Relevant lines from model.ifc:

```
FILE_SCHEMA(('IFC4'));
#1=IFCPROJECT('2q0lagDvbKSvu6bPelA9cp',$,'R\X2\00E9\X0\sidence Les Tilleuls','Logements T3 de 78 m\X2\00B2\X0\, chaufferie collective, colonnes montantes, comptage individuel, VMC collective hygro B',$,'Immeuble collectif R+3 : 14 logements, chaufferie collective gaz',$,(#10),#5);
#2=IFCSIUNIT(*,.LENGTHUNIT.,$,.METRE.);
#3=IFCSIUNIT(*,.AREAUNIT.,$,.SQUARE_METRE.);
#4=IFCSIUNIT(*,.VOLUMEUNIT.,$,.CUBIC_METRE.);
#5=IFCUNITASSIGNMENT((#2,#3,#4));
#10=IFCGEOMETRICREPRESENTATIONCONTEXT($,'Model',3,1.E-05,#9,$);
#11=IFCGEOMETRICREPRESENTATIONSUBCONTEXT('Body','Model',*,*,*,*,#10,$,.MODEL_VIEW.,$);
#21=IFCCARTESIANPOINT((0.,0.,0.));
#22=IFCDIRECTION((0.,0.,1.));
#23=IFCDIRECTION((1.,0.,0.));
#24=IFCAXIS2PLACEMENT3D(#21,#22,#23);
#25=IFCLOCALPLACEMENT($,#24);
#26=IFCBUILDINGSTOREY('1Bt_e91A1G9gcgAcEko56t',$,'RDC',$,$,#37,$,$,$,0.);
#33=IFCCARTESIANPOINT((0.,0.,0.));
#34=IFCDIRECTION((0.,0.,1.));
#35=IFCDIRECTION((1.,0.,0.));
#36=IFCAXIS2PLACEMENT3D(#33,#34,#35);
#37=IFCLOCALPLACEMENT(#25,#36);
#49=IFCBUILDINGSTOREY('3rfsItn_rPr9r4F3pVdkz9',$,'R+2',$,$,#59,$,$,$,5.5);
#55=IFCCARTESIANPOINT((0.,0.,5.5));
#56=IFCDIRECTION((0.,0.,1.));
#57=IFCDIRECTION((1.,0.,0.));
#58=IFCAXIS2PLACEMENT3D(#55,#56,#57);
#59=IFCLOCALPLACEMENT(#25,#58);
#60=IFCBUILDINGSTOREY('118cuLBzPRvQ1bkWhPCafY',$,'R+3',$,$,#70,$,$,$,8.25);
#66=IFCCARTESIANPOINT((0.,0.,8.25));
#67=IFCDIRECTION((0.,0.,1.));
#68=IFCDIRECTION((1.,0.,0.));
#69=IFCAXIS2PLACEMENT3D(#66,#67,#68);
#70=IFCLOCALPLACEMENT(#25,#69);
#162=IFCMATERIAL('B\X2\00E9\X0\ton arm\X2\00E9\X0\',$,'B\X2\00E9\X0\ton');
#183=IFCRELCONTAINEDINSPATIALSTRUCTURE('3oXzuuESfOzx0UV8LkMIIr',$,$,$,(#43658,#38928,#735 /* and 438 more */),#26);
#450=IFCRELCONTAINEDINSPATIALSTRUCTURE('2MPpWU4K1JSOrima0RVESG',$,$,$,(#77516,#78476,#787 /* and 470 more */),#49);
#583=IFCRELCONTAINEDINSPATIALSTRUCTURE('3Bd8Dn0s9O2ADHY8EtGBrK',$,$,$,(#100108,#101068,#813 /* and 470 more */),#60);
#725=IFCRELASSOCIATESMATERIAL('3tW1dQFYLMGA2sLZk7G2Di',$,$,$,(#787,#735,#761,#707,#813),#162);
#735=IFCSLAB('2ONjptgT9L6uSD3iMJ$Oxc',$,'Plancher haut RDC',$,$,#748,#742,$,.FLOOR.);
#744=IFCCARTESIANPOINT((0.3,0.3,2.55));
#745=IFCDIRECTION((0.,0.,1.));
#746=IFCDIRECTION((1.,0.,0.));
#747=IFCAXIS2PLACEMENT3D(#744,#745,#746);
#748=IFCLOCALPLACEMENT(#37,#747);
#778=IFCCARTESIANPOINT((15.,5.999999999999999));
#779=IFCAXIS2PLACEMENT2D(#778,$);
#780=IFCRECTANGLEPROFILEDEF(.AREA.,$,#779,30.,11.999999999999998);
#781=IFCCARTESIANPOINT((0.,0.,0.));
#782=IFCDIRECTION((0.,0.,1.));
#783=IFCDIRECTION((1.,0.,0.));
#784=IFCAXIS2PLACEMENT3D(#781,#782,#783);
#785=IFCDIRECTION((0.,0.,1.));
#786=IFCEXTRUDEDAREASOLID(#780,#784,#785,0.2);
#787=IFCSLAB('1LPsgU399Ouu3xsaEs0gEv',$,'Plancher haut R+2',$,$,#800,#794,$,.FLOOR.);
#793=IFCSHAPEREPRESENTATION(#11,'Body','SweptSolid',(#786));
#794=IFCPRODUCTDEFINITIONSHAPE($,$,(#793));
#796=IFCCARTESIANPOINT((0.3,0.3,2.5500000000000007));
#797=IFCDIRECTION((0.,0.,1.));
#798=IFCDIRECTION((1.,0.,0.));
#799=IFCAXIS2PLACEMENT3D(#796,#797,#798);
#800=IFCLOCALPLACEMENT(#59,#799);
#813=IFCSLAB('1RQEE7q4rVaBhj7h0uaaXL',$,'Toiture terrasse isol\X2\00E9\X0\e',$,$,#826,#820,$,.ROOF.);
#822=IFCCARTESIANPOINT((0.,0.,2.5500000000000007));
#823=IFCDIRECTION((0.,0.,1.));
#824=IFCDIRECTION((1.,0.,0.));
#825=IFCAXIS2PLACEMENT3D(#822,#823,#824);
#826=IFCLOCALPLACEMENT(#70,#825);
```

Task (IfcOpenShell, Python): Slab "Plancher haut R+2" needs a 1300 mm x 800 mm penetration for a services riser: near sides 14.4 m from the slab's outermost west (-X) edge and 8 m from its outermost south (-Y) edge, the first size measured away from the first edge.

```python
import numpy as np
import ifcopenshell
import ifcopenshell.api.feature
import ifcopenshell.api.geometry
import ifcopenshell.api.root
import ifcopenshell.geom
import ifcopenshell.util.placement
import ifcopenshell.util.representation
import ifcopenshell.util.shape
import ifcopenshell.util.unit

model = ifcopenshell.open("model.ifc")
unit_scale = ifcopenshell.util.unit.calculate_unit_scale(model)
settings = ifcopenshell.geom.settings()


def volume(element):
    """Net volume in cubic metres, openings subtracted."""
    shape = ifcopenshell.geom.create_shape(settings, element)
    return ifcopenshell.util.shape.get_volume(shape.geometry)


slab = model.by_id(787)
before = volume(slab)

# Extent in the slab's own axes, in metres. The edges named are its -X and -Y sides.
slab_shape = ifcopenshell.geom.create_shape(settings, slab)
vertices = ifcopenshell.util.shape.get_vertices(slab_shape.geometry)
x_min, y_min, bottom = vertices.min(axis=0)
top = vertices[:, 2].max()

opening = ifcopenshell.api.root.create_entity(model, ifc_class="IfcOpeningElement", name="Services riser opening", predefined_type="OPENING")
context = ifcopenshell.util.representation.get_context(model, "Model", "Body", "MODEL_VIEW")
width, depth = 1.3, 0.8
outline = [(0.0, 0.0), (width, 0.0), (width, depth), (0.0, depth), (0.0, 0.0)]
# Overshoot both faces by 50 mm so the cut is clean.
shape = ifcopenshell.api.geometry.add_slab_representation(
    model, context=context, depth=top - bottom + 0.1, polyline=outline
)
ifcopenshell.api.geometry.assign_representation(model, product=opening, representation=shape)

matrix = ifcopenshell.util.placement.get_local_placement(slab.ObjectPlacement)
matrix[:, 3] = matrix @ np.append(np.array([x_min + 14.4, y_min + 8, bottom - 0.05]) / unit_scale, 1.0)
ifcopenshell.api.geometry.edit_object_placement(model, product=opening, matrix=matrix, is_si=False)
ifcopenshell.api.feature.add_feature(model, feature=opening, element=slab)

after = volume(slab)

print(f"slab volume {before:.3f} -> {after:.3f} m3")

model.write("model_edited.ifc")
```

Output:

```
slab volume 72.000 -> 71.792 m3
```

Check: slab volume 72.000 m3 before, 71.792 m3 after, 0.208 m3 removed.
